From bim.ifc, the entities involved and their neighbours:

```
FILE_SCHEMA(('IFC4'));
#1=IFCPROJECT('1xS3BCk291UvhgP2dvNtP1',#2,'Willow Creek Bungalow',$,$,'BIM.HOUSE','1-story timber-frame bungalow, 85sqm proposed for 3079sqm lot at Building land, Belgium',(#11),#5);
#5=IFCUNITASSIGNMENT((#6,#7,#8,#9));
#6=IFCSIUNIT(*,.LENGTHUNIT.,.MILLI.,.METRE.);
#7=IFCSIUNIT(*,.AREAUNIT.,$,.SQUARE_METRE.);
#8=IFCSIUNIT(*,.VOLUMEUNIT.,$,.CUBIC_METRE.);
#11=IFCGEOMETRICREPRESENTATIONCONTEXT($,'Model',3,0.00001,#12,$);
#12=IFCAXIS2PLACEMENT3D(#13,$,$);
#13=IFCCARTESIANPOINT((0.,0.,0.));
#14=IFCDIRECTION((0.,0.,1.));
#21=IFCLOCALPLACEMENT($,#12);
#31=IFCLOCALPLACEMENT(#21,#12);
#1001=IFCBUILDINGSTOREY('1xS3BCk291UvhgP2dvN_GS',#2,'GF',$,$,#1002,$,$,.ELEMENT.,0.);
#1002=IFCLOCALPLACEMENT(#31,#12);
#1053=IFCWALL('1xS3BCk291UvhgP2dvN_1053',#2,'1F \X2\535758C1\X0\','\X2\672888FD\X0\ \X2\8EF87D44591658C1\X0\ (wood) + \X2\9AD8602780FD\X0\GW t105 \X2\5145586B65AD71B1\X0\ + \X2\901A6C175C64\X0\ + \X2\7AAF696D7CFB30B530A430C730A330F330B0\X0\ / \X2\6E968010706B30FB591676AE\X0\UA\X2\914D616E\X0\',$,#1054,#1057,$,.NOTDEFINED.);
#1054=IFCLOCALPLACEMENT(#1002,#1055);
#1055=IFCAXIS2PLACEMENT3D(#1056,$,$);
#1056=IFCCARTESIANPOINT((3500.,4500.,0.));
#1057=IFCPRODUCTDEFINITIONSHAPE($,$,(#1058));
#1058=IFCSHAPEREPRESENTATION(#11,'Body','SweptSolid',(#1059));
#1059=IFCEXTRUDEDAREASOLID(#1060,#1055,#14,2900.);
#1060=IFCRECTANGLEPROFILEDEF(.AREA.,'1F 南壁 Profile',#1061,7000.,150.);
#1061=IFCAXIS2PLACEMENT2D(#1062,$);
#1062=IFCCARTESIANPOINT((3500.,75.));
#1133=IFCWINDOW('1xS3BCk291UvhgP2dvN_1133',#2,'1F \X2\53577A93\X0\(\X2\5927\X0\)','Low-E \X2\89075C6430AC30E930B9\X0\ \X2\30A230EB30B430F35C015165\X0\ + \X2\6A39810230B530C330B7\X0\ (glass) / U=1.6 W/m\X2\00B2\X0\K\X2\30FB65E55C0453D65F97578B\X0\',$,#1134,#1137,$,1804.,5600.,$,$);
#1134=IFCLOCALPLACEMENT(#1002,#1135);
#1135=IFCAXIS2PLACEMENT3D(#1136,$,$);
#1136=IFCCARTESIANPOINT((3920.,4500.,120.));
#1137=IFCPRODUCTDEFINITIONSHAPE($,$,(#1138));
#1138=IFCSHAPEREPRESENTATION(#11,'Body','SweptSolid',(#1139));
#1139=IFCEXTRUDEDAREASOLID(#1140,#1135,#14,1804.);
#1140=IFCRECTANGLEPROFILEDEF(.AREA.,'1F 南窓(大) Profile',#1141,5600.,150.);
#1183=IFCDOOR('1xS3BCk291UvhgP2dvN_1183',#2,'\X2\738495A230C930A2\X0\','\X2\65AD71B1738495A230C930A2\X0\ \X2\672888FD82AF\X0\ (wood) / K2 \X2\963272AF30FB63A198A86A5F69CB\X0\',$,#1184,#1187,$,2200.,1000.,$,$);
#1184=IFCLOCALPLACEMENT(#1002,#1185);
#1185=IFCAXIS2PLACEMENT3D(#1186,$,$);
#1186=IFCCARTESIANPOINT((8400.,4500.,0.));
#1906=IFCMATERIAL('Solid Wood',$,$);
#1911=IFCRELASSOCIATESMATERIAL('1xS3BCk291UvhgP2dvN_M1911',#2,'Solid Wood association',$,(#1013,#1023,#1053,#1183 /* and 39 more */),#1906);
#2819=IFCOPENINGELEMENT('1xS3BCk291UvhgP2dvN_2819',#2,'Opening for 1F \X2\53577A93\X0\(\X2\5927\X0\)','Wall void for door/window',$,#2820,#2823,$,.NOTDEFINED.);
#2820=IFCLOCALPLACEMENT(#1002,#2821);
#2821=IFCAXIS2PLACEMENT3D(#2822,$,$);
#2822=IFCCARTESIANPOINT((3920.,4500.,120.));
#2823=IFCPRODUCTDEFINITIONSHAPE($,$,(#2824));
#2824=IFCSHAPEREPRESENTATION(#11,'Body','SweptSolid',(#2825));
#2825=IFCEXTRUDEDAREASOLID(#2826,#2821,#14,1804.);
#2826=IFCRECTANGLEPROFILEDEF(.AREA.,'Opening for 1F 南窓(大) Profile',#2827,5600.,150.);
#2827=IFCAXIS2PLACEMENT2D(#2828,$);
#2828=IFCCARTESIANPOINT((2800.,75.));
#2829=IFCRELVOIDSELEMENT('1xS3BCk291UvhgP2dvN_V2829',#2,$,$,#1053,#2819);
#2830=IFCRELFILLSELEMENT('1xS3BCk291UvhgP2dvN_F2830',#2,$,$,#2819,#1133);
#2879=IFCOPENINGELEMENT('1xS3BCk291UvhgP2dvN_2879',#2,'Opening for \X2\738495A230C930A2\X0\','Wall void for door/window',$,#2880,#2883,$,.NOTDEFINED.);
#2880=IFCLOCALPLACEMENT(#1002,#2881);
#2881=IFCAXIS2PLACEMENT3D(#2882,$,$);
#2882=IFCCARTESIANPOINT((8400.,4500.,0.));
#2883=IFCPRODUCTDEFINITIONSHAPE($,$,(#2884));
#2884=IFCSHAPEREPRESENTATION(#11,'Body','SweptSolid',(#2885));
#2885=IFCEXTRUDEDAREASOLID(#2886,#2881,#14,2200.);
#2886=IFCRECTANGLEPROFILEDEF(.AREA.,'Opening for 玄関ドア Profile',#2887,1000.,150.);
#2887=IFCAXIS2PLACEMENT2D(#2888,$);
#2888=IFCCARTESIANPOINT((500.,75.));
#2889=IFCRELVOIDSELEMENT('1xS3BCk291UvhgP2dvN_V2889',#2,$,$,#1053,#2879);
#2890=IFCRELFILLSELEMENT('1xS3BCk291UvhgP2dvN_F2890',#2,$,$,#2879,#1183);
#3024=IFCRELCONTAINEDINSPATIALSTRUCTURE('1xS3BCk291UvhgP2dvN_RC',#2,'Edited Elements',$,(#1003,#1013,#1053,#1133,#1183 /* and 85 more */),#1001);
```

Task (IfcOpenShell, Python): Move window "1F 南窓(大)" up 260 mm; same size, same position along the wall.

```python
import numpy as np
import ifcopenshell
import ifcopenshell.api.geometry
import ifcopenshell.util.placement
import ifcopenshell.util.unit

model = ifcopenshell.open("bim.ifc")
unit_scale = ifcopenshell.util.unit.calculate_unit_scale(model)

window = model.by_guid("1xS3BCk291UvhgP2dvN_1133")
opening = window.FillsVoids[0].RelatingOpeningElement
dz = 0.26 / unit_scale

shift = np.array([0.0, 0.0, dz])
# The window is not placed relative to its opening, so move both.
for product in (opening, window):
    matrix = ifcopenshell.util.placement.get_local_placement(product.ObjectPlacement)
    matrix[:3, 3] += shift
    ifcopenshell.api.geometry.edit_object_placement(model, product=product, matrix=matrix, is_si=False)

print(f"moved by {dz * unit_scale:+.3f} m")

model.write("bim_updated.ifc")
```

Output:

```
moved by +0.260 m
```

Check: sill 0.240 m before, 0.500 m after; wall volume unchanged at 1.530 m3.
